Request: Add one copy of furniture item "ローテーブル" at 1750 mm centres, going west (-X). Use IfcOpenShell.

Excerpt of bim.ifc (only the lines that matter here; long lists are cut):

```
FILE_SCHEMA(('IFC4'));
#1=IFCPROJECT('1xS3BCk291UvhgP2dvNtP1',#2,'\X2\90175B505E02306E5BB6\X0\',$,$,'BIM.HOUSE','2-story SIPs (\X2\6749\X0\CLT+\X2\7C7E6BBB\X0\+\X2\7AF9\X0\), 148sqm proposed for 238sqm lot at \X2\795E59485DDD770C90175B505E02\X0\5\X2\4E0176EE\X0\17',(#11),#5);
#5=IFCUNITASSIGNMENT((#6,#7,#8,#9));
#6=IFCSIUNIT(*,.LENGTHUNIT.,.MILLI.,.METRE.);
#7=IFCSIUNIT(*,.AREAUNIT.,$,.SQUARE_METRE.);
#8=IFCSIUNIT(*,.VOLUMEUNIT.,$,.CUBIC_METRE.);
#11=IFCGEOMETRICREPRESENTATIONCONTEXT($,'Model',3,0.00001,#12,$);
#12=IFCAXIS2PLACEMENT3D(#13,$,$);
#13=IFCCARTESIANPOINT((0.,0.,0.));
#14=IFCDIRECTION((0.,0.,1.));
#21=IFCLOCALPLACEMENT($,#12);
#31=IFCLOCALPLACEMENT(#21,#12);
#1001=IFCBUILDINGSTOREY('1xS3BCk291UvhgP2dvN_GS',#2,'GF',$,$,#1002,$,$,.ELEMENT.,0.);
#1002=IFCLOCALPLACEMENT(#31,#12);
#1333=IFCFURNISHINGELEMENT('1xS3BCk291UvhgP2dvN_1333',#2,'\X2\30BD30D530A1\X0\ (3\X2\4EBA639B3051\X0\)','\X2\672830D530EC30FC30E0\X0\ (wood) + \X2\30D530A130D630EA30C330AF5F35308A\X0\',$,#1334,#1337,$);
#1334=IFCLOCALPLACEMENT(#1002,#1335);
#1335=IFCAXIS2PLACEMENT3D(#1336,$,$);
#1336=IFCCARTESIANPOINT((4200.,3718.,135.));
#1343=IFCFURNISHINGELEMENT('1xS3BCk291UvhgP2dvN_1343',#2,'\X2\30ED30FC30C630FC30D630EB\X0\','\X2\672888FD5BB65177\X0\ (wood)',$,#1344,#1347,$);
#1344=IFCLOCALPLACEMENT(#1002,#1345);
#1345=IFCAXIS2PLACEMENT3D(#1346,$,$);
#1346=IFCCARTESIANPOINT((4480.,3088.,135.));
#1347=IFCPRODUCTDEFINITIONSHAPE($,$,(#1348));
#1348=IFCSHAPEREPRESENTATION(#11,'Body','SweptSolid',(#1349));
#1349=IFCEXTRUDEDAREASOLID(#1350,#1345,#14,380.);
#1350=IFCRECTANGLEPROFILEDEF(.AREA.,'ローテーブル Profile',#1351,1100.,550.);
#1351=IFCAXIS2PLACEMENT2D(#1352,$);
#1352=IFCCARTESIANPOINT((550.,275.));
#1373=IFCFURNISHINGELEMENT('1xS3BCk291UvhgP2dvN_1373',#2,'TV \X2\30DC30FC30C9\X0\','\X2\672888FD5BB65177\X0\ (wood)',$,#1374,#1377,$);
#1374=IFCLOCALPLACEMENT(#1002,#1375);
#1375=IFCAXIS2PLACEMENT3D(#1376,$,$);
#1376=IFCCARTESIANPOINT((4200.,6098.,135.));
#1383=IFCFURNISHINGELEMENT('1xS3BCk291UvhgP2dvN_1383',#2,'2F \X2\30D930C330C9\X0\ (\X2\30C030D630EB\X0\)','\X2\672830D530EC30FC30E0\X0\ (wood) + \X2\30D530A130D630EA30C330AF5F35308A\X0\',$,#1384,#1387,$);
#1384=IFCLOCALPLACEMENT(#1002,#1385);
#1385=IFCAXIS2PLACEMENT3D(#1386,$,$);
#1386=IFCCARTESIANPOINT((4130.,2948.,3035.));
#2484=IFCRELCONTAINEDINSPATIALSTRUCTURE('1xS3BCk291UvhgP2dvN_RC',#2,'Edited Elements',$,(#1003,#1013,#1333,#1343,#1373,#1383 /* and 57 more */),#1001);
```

```python
import numpy as np
import ifcopenshell
import ifcopenshell.api.geometry
import ifcopenshell.api.root
import ifcopenshell.util.element
import ifcopenshell.util.placement

model = ifcopenshell.open("bim.ifc")


def reuse_history(source, copy):
    """copy_class also copies each property set's owner history, people and application; keep the originals."""
    for rel in copy.IsDefinedBy:
        if rel.is_a("IfcRelDefinesByProperties") and (history := rel.RelatingPropertyDefinition.OwnerHistory):
            rel.RelatingPropertyDefinition.OwnerHistory = source.OwnerHistory
            ifcopenshell.util.element.remove_deep2(model, history)


source = model.by_guid("1xS3BCk291UvhgP2dvN_1343")
base = ifcopenshell.util.placement.get_local_placement(source.ObjectPlacement)
step = np.array([-1.0, 0.0, 0.0]) * 1750.0

for i in range(1, 2):
    copy = ifcopenshell.api.root.copy_class(model, product=source)
    copy.Representation = ifcopenshell.util.element.copy_deep(
        model, source.Representation, exclude=["IfcGeometricRepresentationContext", "IfcRepresentationMap"]
    )
    reuse_history(source, copy)
    matrix = base.copy()
    matrix[:3, 3] += i * step
    print("added at", matrix[:3, 3].round(3) + 0.0)
    ifcopenshell.api.geometry.edit_object_placement(model, product=copy, matrix=matrix, is_si=False)

model.write("bim_v2.ifc")
```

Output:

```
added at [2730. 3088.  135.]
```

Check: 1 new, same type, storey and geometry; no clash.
